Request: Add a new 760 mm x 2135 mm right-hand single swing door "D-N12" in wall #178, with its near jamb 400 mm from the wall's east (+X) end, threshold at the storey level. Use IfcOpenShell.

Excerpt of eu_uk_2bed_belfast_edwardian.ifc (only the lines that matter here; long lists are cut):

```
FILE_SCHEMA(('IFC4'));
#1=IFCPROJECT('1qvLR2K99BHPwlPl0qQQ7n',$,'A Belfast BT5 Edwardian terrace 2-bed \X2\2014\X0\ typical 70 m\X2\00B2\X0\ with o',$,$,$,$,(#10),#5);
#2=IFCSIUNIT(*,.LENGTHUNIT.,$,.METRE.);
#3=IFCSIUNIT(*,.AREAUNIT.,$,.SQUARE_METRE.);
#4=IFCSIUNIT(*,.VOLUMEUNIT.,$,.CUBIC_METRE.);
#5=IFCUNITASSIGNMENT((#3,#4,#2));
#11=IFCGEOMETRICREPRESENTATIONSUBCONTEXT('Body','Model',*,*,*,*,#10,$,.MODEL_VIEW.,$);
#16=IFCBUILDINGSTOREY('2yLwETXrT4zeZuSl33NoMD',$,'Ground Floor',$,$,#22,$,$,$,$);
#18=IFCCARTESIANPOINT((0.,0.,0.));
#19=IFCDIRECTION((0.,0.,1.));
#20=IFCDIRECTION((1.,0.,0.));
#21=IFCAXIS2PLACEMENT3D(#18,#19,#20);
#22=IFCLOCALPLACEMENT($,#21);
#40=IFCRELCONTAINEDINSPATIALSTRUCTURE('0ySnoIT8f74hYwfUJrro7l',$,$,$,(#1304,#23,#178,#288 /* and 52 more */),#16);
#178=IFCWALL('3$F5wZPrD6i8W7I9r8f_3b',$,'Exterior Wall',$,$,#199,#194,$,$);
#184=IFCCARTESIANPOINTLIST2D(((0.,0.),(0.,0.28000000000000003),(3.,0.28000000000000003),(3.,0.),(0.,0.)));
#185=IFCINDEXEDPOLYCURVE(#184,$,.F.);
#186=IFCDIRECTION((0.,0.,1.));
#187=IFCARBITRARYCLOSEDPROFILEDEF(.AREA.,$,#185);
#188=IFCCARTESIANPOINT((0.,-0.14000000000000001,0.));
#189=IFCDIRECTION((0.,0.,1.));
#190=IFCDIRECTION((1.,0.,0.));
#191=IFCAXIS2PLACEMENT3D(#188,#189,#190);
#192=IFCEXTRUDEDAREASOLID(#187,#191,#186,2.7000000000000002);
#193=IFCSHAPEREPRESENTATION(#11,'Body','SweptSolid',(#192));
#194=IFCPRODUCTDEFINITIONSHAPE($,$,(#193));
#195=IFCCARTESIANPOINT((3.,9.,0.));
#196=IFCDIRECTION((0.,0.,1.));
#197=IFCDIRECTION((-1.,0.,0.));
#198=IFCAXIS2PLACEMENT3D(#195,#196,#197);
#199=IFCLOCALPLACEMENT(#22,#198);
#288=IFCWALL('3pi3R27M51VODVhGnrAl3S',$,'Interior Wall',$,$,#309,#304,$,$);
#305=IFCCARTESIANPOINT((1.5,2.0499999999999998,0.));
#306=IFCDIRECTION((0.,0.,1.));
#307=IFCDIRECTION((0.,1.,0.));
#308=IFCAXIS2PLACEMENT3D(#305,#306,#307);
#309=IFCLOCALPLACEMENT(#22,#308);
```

```python
import numpy as np
import ifcopenshell
import ifcopenshell.api.feature
import ifcopenshell.api.geometry
import ifcopenshell.api.root
import ifcopenshell.api.spatial
import ifcopenshell.geom
import ifcopenshell.util.element
import ifcopenshell.util.placement
import ifcopenshell.util.representation
import ifcopenshell.util.shape
import ifcopenshell.util.unit

model = ifcopenshell.open("eu_uk_2bed_belfast_edwardian.ifc")
unit_scale = ifcopenshell.util.unit.calculate_unit_scale(model)
settings = ifcopenshell.geom.settings()


def volume(element):
    """Net volume in cubic metres, openings subtracted."""
    shape = ifcopenshell.geom.create_shape(settings, element)
    return ifcopenshell.util.shape.get_volume(shape.geometry)


wall = model.by_guid("3$F5wZPrD6i8W7I9r8f_3b")
storey = ifcopenshell.util.element.get_container(wall, ifc_class="IfcBuildingStorey")
context = ifcopenshell.util.representation.get_context(model, "Model", "Body", "MODEL_VIEW")
before = volume(wall)

width, height, from_end, sill = 0.76, 2.135, 0.4, 0.0  # metres

# The wall runs along its own X axis, and the end named is its -X end.
wall_shape = ifcopenshell.geom.create_shape(settings, wall)
x, y, z = ifcopenshell.util.shape.get_vertices(wall_shape.geometry).T
start = x.min() + from_end
face, thickness = float(y.min()), float(y.max() - y.min())
wall_matrix = ifcopenshell.util.placement.get_local_placement(wall.ObjectPlacement)
level = ifcopenshell.util.placement.get_local_placement(storey.ObjectPlacement)[2, 3]


def in_wall(x, y):
    """Placement at x, y metres in the wall's axes, at sill height."""
    matrix = wall_matrix.copy()
    matrix[:, 3] = wall_matrix @ np.array([x / unit_scale, y / unit_scale, 0.0, 1.0])
    matrix[2, 3] = level + sill / unit_scale
    return matrix


# Opening: a box that overshoots both wall faces by 50 mm.
opening = ifcopenshell.api.root.create_entity(model, ifc_class="IfcOpeningElement", predefined_type="OPENING")
box = ifcopenshell.api.geometry.add_wall_representation(
    model, context=context, length=width, height=height, thickness=thickness + 0.1
)
ifcopenshell.api.geometry.assign_representation(model, product=opening, representation=box)
ifcopenshell.api.geometry.edit_object_placement(model, product=opening, matrix=in_wall(start, face - 0.05), is_si=False)
ifcopenshell.api.feature.add_feature(model, feature=opening, element=wall)

door = ifcopenshell.api.root.create_entity(model, ifc_class="IfcDoor", name="D-N12", predefined_type="DOOR")
door.OverallWidth, door.OverallHeight = width / unit_scale, height / unit_scale
door.OperationType = "SINGLE_SWING_RIGHT"
body = ifcopenshell.api.geometry.add_door_representation(
    model,
    context=context,
    overall_width=door.OverallWidth,
    overall_height=door.OverallHeight,
    operation_type="SINGLE_SWING_RIGHT",
    lining_properties={"LiningDepth": thickness / unit_scale, "ThresholdDepth": thickness / unit_scale},
)
ifcopenshell.api.geometry.assign_representation(model, product=door, representation=body)
ifcopenshell.api.spatial.assign_container(model, products=[door], relating_structure=storey)
ifcopenshell.api.feature.add_filling(model, opening=opening, element=door)

# The lining spans the wall, so the door starts at the wall face.
ifcopenshell.api.geometry.edit_object_placement(model, product=door, matrix=in_wall(start, face), is_si=False)

after = volume(wall)

print(f"wall volume {before:.3f} -> {after:.3f} m3")

model.write("eu_uk_2bed_belfast_edwardian_v2.ifc")
```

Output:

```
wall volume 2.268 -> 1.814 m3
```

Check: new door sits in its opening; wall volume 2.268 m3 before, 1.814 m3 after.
